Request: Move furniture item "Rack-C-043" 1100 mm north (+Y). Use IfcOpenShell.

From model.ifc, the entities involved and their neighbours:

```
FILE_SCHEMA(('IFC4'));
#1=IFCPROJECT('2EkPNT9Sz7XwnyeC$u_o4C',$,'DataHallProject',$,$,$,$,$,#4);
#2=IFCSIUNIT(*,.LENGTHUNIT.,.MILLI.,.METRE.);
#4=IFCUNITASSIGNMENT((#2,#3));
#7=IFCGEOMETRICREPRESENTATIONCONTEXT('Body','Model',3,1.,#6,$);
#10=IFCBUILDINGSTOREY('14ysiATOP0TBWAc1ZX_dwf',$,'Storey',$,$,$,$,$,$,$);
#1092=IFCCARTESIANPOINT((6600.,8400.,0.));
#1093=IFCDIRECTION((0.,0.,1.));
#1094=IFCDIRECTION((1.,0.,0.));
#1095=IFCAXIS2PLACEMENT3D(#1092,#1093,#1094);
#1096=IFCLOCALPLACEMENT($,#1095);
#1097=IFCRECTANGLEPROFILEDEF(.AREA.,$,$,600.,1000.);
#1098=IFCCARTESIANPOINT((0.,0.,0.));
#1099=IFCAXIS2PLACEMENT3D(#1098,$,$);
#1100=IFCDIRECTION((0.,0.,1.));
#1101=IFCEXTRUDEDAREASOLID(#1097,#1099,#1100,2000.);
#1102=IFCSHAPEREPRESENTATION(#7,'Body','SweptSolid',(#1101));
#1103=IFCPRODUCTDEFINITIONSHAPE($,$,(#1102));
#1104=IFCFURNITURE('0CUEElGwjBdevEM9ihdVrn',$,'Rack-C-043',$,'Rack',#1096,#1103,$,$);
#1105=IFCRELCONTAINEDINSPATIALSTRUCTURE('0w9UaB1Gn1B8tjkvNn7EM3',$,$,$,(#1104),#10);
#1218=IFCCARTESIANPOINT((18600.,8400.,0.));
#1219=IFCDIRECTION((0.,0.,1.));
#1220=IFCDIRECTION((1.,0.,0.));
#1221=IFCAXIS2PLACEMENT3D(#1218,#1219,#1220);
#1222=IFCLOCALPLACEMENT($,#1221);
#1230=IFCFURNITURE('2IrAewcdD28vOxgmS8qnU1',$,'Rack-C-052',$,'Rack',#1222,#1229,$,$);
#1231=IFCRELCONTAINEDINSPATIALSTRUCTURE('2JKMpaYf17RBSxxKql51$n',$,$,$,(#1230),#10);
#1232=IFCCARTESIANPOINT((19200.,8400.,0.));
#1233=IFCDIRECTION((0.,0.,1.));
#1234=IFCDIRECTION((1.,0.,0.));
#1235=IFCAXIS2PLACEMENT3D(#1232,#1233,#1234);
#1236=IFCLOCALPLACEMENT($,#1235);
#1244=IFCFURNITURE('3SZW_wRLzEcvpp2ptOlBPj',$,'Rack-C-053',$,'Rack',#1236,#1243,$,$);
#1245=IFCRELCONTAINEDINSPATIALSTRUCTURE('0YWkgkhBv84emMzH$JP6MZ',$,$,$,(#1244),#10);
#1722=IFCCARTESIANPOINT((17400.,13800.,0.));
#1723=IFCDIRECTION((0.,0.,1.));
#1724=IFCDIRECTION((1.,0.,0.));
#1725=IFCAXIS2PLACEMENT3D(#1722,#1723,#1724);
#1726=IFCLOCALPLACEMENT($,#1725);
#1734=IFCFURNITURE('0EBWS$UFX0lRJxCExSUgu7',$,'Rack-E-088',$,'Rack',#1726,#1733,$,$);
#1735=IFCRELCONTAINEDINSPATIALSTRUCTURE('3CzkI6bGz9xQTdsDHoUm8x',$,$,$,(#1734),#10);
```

```python
import ifcopenshell
import ifcopenshell.api.geometry
import ifcopenshell.util.placement
import ifcopenshell.util.unit

model = ifcopenshell.open("model.ifc")
unit_scale = ifcopenshell.util.unit.calculate_unit_scale(model)

item = model.by_id(1104)
matrix = ifcopenshell.util.placement.get_local_placement(item.ObjectPlacement)
matrix[1, 3] += 1.1 / unit_scale
ifcopenshell.api.geometry.edit_object_placement(model, product=item, matrix=matrix, is_si=False)

print(ifcopenshell.util.placement.get_local_placement(item.ObjectPlacement).round(3) + 0.0)

model.write("model_rev.ifc")
```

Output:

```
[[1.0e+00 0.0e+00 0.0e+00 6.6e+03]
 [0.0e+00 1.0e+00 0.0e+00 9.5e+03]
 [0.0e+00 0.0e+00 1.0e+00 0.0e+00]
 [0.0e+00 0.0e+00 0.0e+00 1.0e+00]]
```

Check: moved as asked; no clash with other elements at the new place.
